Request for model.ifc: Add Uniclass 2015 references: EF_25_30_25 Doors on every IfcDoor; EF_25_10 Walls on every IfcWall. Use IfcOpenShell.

First a look at what the model holds.

```python
import ifcopenshell

model = ifcopenshell.open("model.ifc")
print(model.schema)
print("classifications:", [c.Name for c in model.by_type("IfcClassification")])
for ifc_class in ("IfcDoor", "IfcRoof", "IfcStair", "IfcWall", "IfcWindow"):
    print(ifc_class, len(model.by_type(ifc_class)))
```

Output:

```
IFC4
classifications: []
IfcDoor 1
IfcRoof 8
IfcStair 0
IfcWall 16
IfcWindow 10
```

```python
import ifcopenshell
import ifcopenshell.api.classification

model = ifcopenshell.open("model.ifc")

system = ifcopenshell.api.classification.add_classification(model, classification="Uniclass 2015")

codes = {
    "IfcDoor": ("EF_25_30_25", "Doors"),
    "IfcWall": ("EF_25_10", "Walls"),
}
for ifc_class, (code, name) in codes.items():
    products = model.by_type(ifc_class)
    ifcopenshell.api.classification.add_reference(
        model, products=products, classification=system, identification=code, name=name
    )
    print(code, len(products))

model.write("model-out.ifc")
```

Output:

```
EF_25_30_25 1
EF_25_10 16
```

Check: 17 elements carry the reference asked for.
